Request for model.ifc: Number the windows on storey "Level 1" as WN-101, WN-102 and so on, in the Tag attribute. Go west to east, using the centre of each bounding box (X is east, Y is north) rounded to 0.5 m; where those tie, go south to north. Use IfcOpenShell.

First a look at what the model holds.

```python
import ifcopenshell
import ifcopenshell.util.element
import ifcopenshell.util.placement

model = ifcopenshell.open("model.ifc")
print(model.schema)
storey = next(s for s in model.by_type("IfcBuildingStorey") if s.Name == "Level 1")
windows = [e for e in ifcopenshell.util.element.get_decomposition(storey) if e.is_a("IfcWindow")]
for e in sorted(windows, key=lambda e: e.id()):
    origin = ifcopenshell.util.placement.get_local_placement(e.ObjectPlacement)[:3, 3]
    print(e.id(), e.Tag, e.Name, origin.round(2) + 0.0, sep=" | ")
```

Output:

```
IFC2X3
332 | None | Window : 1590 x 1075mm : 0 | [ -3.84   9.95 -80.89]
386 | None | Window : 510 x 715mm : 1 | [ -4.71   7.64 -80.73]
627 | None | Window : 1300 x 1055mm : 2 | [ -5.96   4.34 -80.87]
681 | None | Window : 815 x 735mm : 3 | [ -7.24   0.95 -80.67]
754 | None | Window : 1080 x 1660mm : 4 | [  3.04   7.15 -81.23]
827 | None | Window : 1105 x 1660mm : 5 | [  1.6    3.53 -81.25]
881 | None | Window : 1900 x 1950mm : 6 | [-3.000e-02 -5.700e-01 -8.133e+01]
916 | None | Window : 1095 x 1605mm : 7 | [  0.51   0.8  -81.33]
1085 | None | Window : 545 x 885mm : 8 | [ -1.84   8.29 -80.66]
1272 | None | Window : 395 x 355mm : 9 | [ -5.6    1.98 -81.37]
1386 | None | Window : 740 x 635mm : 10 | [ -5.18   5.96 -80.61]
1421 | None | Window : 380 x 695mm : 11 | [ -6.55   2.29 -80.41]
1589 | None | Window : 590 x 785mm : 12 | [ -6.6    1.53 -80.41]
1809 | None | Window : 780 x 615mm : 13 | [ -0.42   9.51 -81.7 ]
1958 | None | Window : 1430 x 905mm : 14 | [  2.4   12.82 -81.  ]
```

```python
import ifcopenshell
import ifcopenshell.geom
import ifcopenshell.util.element
import ifcopenshell.util.shape

model = ifcopenshell.open("model.ifc")
settings = ifcopenshell.geom.settings()
settings.set("use-world-coords", True)


def centre(element):
    shape = ifcopenshell.geom.create_shape(settings, element)
    return ifcopenshell.util.shape.get_bbox_centroid(shape.geometry)


storey = next(s for s in model.by_type("IfcBuildingStorey") if s.Name == "Level 1")
windows = [e for e in ifcopenshell.util.element.get_decomposition(storey) if e.is_a("IfcWindow")]

# Insertion points can sit at a corner or the storey origin, so sort by the geometry (in metres).
centres = {e: centre(e) for e in windows}
windows.sort(key=lambda e: (round(centres[e][0] / 0.5), centres[e][1]))

for i, e in enumerate(windows, start=1):
    number = f"WN-1{i:02d}"
    e.Tag = number
    print(e.id(), number)

model.write("model_updated.ifc")
```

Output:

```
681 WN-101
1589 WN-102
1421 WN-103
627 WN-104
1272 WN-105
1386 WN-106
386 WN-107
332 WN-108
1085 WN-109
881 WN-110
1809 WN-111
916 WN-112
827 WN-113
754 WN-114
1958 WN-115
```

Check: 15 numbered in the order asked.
